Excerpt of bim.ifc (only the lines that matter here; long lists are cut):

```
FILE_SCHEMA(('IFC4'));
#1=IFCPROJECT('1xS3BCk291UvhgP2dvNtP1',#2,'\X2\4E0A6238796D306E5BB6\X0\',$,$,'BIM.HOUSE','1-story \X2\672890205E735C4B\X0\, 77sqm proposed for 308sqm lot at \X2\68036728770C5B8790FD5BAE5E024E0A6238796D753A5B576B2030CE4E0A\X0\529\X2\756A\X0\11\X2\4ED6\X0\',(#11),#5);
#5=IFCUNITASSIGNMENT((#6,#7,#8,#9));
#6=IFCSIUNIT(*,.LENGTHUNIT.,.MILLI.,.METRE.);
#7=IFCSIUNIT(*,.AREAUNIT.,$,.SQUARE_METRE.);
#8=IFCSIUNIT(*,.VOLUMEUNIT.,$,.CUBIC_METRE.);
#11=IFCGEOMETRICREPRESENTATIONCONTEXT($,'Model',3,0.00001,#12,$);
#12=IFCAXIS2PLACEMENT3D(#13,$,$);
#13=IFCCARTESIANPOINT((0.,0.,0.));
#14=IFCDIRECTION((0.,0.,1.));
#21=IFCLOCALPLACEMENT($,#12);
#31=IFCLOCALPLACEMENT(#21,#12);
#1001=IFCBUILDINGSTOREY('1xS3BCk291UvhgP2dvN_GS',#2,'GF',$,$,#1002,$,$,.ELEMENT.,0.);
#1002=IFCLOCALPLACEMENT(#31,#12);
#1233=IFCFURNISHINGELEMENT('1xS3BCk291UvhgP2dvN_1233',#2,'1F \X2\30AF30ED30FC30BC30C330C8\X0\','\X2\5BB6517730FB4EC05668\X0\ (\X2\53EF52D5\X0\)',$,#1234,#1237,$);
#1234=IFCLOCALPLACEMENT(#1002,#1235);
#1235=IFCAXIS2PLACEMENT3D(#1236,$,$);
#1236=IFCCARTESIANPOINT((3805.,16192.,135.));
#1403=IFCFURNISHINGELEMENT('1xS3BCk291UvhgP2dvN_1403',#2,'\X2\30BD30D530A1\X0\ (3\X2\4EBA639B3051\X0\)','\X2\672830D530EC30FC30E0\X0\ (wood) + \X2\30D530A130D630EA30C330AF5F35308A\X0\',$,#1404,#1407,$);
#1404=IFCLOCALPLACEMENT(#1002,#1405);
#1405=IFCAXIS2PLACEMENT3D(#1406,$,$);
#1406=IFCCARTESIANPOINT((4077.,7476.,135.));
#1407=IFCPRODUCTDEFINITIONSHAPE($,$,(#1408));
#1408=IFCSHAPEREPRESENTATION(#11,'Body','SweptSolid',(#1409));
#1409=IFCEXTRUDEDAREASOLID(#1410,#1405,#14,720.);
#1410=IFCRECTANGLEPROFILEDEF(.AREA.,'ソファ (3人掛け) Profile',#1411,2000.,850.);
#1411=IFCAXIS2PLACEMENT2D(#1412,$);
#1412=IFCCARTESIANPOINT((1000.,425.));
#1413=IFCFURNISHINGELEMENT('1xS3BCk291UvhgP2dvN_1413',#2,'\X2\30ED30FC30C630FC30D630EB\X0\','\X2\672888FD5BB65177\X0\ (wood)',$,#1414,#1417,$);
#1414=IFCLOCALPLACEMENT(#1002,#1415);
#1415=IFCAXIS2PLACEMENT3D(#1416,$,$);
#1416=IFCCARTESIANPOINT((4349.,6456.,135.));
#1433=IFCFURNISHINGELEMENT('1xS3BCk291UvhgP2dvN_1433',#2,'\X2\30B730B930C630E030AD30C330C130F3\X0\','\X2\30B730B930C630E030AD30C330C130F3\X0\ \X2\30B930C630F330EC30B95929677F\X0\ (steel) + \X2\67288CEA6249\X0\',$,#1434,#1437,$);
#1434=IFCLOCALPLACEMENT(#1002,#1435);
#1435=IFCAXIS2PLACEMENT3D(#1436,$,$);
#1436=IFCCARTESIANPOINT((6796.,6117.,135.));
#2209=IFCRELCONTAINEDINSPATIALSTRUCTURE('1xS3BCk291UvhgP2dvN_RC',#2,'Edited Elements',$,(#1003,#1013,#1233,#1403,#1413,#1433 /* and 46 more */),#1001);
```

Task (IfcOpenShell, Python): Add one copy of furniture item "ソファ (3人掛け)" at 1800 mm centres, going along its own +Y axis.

```python
import ifcopenshell
import ifcopenshell.api.geometry
import ifcopenshell.api.root
import ifcopenshell.util.element
import ifcopenshell.util.placement

model = ifcopenshell.open("bim.ifc")


def reuse_history(source, copy):
    """copy_class also copies each property set's owner history, people and application; keep the originals."""
    for rel in copy.IsDefinedBy:
        if rel.is_a("IfcRelDefinesByProperties") and (history := rel.RelatingPropertyDefinition.OwnerHistory):
            rel.RelatingPropertyDefinition.OwnerHistory = source.OwnerHistory
            ifcopenshell.util.element.remove_deep2(model, history)


source = model.by_guid("1xS3BCk291UvhgP2dvN_1403")
base = ifcopenshell.util.placement.get_local_placement(source.ObjectPlacement)
step = base[:3, 1] * 1800.0

for i in range(1, 2):
    copy = ifcopenshell.api.root.copy_class(model, product=source)
    copy.Representation = ifcopenshell.util.element.copy_deep(
        model, source.Representation, exclude=["IfcGeometricRepresentationContext", "IfcRepresentationMap"]
    )
    reuse_history(source, copy)
    matrix = base.copy()
    matrix[:3, 3] += i * step
    print("added at", matrix[:3, 3].round(3) + 0.0)
    ifcopenshell.api.geometry.edit_object_placement(model, product=copy, matrix=matrix, is_si=False)

model.write("bim-out.ifc")
```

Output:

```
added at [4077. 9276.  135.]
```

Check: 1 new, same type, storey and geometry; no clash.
